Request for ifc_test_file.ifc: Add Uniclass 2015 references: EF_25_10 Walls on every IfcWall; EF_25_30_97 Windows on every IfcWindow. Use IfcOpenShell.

First a look at what the model holds.

```python
import ifcopenshell

model = ifcopenshell.open("ifc_test_file.ifc")
print(model.schema)
print("classifications:", [c.Name for c in model.by_type("IfcClassification")])
for ifc_class in ("IfcDoor", "IfcRoof", "IfcStair", "IfcWall", "IfcWindow"):
    print(ifc_class, len(model.by_type(ifc_class)))
```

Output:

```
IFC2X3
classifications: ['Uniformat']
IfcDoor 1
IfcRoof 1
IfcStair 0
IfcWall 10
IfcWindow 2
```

```python
import ifcopenshell
import ifcopenshell.api.classification

model = ifcopenshell.open("ifc_test_file.ifc")

# IFC2X3 requires Source and Edition and has no link from the project to the system.
system = model.create_entity("IfcClassification", Source="NBS", Edition="2015", Name="Uniclass 2015")

codes = {
    "IfcWall": ("EF_25_10", "Walls"),
    "IfcWindow": ("EF_25_30_97", "Windows"),
}
for ifc_class, (code, name) in codes.items():
    products = model.by_type(ifc_class)
    ifcopenshell.api.classification.add_reference(
        model, products=products, classification=system, identification=code, name=name
    )
    print(code, len(products))

model.write("ifc_test_file_updated.ifc")
```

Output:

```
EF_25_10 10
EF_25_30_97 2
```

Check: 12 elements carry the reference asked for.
